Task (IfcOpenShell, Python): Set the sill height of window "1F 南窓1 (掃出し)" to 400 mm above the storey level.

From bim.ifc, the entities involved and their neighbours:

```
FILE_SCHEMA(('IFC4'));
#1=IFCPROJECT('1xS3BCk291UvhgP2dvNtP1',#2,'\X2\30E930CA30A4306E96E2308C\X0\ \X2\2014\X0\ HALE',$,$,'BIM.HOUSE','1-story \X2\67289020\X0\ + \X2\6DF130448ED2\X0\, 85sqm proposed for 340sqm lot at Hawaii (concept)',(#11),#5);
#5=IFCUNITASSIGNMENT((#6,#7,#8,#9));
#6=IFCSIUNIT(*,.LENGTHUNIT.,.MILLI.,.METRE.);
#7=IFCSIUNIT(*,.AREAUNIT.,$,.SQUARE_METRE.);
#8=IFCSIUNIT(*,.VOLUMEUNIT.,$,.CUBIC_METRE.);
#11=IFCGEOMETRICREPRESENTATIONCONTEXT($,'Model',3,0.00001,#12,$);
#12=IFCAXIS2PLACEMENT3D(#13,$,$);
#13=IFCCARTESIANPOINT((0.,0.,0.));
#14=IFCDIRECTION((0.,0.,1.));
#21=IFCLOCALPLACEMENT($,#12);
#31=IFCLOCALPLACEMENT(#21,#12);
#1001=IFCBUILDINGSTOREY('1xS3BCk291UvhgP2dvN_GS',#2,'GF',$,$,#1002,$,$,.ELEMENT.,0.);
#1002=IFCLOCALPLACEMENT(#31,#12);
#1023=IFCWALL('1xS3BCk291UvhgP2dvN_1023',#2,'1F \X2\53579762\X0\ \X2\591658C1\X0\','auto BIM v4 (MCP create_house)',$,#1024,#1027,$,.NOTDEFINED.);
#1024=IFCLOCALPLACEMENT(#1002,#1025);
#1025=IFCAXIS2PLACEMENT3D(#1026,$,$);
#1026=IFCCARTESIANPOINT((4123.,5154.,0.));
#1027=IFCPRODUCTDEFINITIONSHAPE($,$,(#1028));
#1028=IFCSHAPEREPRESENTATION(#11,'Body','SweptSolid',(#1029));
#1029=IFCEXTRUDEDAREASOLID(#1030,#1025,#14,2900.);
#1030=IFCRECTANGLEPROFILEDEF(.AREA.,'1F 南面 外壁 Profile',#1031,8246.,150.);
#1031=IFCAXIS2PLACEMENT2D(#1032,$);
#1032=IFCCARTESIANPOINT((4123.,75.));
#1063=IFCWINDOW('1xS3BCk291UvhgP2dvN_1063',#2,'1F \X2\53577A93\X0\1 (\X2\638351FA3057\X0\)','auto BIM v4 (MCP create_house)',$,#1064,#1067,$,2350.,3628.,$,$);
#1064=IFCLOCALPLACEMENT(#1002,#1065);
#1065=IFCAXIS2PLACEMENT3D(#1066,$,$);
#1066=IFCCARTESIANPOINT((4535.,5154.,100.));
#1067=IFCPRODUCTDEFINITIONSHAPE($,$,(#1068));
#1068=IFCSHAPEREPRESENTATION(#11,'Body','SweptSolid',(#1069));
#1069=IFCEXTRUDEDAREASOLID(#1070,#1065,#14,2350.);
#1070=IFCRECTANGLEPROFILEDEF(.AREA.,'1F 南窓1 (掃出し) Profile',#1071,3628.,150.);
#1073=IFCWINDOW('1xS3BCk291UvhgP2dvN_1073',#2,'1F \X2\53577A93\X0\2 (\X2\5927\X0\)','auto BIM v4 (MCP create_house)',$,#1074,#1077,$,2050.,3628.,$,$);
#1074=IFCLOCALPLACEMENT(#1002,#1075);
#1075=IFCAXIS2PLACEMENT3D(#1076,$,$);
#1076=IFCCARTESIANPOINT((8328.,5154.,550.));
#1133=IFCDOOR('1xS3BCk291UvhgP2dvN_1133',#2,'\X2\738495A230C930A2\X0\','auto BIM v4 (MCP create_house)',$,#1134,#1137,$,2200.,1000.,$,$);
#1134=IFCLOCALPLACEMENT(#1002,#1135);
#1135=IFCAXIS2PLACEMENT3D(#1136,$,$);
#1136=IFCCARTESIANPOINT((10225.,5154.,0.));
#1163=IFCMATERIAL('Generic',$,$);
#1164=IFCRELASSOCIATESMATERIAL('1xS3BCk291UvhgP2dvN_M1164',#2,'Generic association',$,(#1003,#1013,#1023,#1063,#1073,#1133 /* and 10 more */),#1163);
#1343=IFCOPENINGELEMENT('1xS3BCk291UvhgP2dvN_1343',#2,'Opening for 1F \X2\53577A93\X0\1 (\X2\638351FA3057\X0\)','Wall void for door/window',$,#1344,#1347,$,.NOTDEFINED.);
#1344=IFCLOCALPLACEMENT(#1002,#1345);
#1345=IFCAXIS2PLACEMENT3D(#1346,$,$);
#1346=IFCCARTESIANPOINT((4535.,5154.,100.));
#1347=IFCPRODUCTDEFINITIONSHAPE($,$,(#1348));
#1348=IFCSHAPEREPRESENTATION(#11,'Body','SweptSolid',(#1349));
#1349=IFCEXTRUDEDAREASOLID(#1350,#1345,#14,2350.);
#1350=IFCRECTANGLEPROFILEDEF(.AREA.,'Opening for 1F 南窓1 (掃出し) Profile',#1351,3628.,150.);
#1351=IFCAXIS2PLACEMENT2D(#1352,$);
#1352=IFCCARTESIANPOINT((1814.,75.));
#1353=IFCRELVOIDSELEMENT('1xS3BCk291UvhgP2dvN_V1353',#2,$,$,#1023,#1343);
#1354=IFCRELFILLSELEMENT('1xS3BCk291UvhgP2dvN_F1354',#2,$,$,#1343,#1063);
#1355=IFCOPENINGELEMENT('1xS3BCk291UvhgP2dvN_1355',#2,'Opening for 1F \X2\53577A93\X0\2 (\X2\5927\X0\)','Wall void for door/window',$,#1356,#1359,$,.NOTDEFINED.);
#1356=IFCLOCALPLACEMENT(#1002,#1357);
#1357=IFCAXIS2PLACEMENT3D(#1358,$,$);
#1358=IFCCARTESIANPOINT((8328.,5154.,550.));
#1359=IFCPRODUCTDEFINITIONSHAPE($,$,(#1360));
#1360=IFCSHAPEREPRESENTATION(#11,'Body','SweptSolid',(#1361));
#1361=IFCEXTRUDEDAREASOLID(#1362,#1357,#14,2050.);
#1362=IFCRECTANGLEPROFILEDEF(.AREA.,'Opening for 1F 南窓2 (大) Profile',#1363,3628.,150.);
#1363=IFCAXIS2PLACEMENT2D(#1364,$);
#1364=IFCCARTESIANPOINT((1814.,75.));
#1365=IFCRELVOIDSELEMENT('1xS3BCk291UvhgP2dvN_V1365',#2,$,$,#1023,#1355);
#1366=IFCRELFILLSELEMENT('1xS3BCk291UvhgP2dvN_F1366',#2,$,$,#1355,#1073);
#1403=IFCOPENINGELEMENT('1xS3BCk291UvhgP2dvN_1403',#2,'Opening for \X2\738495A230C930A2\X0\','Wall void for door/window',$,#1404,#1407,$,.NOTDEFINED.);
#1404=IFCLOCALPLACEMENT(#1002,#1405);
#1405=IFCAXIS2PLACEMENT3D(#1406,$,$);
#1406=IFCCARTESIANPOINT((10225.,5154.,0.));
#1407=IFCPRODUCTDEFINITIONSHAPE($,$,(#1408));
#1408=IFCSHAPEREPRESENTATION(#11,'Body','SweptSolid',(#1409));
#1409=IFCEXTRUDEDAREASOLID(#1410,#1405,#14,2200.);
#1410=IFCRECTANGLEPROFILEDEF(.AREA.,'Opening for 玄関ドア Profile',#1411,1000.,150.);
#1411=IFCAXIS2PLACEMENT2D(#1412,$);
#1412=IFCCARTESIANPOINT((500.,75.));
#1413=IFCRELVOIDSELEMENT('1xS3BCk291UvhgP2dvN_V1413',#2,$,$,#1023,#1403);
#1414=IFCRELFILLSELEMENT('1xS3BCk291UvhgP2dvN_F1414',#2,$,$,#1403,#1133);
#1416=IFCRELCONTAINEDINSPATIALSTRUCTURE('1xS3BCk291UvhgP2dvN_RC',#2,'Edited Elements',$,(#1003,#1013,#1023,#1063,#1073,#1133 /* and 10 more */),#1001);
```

```python
import numpy as np
import ifcopenshell
import ifcopenshell.api.geometry
import ifcopenshell.geom
import ifcopenshell.util.element
import ifcopenshell.util.placement
import ifcopenshell.util.shape
import ifcopenshell.util.unit

model = ifcopenshell.open("bim.ifc")
unit_scale = ifcopenshell.util.unit.calculate_unit_scale(model)

window = model.by_guid("1xS3BCk291UvhgP2dvN_1063")
opening = window.FillsVoids[0].RelatingOpeningElement
storey = ifcopenshell.util.element.get_container(window, ifc_class="IfcBuildingStorey")
level = ifcopenshell.util.placement.get_local_placement(storey.ObjectPlacement)[2, 3]

# The opening's origin need not be at the sill, so measure its lowest point.
shape = ifcopenshell.geom.create_shape(ifcopenshell.geom.settings(), opening)
bottom = ifcopenshell.util.shape.get_shape_bottom_elevation(shape, shape.geometry) / unit_scale
dz = level + 0.4 / unit_scale - bottom

shift = np.array([0.0, 0.0, dz])
# The window is not placed relative to its opening, so move both.
for product in (opening, window):
    matrix = ifcopenshell.util.placement.get_local_placement(product.ObjectPlacement)
    matrix[:3, 3] += shift
    ifcopenshell.api.geometry.edit_object_placement(model, product=product, matrix=matrix, is_si=False)

print(f"moved by {dz * unit_scale:+.3f} m")

model.write("bim-out.ifc")
```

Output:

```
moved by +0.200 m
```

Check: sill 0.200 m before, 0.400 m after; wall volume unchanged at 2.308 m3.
